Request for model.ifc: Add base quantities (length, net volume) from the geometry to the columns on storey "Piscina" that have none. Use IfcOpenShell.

First a look at what the model holds.

```python
import ifcopenshell
import ifcopenshell.util.element
import ifcopenshell.util.unit

model = ifcopenshell.open("model.ifc")
print(model.schema)
for unit_type in ("LENGTHUNIT", "AREAUNIT", "VOLUMEUNIT"):
    print(unit_type, ifcopenshell.util.unit.calculate_unit_scale(model, unit_type))
storey = next(s for s in model.by_type("IfcBuildingStorey") if s.Name == "Piscina")
columns = [e for e in ifcopenshell.util.element.get_decomposition(storey) if e.is_a("IfcColumn")]
for e in sorted(columns, key=lambda e: e.id()):
    print(e.id(), e.is_a(), e.Name, list(ifcopenshell.util.element.get_psets(e, qtos_only=True)), sep=" | ")
```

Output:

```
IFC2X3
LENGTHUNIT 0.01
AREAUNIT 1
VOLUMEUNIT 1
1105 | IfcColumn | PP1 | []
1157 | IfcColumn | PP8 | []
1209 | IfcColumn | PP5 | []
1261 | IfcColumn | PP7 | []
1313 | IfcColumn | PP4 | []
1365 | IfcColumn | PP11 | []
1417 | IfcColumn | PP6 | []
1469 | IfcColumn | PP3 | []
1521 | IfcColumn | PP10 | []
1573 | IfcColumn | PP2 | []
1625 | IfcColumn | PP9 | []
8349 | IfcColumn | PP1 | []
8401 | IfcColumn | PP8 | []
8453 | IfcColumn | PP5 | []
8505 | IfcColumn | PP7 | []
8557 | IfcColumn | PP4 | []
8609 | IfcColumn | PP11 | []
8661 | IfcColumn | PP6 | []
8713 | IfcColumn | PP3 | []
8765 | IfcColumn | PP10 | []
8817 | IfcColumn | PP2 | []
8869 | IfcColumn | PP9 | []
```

```python
import ifcopenshell
import ifcopenshell.api.pset
import ifcopenshell.geom
import ifcopenshell.util.element
import ifcopenshell.util.shape
import ifcopenshell.util.unit

model = ifcopenshell.open("model.ifc")
unit_scale = ifcopenshell.util.unit.calculate_unit_scale(model)
volume_scale = ifcopenshell.util.unit.calculate_unit_scale(model, "VOLUMEUNIT")
settings = ifcopenshell.geom.settings()

storey = next(s for s in model.by_type("IfcBuildingStorey") if s.Name == "Piscina")
columns = [e for e in ifcopenshell.util.element.get_decomposition(storey) if e.is_a("IfcColumn")]

for e in sorted(columns, key=lambda e: e.id()):
    if ifcopenshell.util.element.get_psets(e, qtos_only=True, should_inherit=False):
        continue
    # Geometry comes back in metres, in the element's own axes.
    shape = ifcopenshell.geom.create_shape(settings, e)
    values = {
        "Length": ifcopenshell.util.shape.get_z(shape.geometry) / unit_scale,
        "NetVolume": ifcopenshell.util.shape.get_volume(shape.geometry) / volume_scale,
    }
    qto = ifcopenshell.api.pset.add_qto(model, product=e, name="BaseQuantities")
    ifcopenshell.api.pset.edit_qto(model, qto=qto, properties=values)
    print(e.id(), {k: round(v, 3) for k, v in values.items()})

model.write("model_edited.ifc")
```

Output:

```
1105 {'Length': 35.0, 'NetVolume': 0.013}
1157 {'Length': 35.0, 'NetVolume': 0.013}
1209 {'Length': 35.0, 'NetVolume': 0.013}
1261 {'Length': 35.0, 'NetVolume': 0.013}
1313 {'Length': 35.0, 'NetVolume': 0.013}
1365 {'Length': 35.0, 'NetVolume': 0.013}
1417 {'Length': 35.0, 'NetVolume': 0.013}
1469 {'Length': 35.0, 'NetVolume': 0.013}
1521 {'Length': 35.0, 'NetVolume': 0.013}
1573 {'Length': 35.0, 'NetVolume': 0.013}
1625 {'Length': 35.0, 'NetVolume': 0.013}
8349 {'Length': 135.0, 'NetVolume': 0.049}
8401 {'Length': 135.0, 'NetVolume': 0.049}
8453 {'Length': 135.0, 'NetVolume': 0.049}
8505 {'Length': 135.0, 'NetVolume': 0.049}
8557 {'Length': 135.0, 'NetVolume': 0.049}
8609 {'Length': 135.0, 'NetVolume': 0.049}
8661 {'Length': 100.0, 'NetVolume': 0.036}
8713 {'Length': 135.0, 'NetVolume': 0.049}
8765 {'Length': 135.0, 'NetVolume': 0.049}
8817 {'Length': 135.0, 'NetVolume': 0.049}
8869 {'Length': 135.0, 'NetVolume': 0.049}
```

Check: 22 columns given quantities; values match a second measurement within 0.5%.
